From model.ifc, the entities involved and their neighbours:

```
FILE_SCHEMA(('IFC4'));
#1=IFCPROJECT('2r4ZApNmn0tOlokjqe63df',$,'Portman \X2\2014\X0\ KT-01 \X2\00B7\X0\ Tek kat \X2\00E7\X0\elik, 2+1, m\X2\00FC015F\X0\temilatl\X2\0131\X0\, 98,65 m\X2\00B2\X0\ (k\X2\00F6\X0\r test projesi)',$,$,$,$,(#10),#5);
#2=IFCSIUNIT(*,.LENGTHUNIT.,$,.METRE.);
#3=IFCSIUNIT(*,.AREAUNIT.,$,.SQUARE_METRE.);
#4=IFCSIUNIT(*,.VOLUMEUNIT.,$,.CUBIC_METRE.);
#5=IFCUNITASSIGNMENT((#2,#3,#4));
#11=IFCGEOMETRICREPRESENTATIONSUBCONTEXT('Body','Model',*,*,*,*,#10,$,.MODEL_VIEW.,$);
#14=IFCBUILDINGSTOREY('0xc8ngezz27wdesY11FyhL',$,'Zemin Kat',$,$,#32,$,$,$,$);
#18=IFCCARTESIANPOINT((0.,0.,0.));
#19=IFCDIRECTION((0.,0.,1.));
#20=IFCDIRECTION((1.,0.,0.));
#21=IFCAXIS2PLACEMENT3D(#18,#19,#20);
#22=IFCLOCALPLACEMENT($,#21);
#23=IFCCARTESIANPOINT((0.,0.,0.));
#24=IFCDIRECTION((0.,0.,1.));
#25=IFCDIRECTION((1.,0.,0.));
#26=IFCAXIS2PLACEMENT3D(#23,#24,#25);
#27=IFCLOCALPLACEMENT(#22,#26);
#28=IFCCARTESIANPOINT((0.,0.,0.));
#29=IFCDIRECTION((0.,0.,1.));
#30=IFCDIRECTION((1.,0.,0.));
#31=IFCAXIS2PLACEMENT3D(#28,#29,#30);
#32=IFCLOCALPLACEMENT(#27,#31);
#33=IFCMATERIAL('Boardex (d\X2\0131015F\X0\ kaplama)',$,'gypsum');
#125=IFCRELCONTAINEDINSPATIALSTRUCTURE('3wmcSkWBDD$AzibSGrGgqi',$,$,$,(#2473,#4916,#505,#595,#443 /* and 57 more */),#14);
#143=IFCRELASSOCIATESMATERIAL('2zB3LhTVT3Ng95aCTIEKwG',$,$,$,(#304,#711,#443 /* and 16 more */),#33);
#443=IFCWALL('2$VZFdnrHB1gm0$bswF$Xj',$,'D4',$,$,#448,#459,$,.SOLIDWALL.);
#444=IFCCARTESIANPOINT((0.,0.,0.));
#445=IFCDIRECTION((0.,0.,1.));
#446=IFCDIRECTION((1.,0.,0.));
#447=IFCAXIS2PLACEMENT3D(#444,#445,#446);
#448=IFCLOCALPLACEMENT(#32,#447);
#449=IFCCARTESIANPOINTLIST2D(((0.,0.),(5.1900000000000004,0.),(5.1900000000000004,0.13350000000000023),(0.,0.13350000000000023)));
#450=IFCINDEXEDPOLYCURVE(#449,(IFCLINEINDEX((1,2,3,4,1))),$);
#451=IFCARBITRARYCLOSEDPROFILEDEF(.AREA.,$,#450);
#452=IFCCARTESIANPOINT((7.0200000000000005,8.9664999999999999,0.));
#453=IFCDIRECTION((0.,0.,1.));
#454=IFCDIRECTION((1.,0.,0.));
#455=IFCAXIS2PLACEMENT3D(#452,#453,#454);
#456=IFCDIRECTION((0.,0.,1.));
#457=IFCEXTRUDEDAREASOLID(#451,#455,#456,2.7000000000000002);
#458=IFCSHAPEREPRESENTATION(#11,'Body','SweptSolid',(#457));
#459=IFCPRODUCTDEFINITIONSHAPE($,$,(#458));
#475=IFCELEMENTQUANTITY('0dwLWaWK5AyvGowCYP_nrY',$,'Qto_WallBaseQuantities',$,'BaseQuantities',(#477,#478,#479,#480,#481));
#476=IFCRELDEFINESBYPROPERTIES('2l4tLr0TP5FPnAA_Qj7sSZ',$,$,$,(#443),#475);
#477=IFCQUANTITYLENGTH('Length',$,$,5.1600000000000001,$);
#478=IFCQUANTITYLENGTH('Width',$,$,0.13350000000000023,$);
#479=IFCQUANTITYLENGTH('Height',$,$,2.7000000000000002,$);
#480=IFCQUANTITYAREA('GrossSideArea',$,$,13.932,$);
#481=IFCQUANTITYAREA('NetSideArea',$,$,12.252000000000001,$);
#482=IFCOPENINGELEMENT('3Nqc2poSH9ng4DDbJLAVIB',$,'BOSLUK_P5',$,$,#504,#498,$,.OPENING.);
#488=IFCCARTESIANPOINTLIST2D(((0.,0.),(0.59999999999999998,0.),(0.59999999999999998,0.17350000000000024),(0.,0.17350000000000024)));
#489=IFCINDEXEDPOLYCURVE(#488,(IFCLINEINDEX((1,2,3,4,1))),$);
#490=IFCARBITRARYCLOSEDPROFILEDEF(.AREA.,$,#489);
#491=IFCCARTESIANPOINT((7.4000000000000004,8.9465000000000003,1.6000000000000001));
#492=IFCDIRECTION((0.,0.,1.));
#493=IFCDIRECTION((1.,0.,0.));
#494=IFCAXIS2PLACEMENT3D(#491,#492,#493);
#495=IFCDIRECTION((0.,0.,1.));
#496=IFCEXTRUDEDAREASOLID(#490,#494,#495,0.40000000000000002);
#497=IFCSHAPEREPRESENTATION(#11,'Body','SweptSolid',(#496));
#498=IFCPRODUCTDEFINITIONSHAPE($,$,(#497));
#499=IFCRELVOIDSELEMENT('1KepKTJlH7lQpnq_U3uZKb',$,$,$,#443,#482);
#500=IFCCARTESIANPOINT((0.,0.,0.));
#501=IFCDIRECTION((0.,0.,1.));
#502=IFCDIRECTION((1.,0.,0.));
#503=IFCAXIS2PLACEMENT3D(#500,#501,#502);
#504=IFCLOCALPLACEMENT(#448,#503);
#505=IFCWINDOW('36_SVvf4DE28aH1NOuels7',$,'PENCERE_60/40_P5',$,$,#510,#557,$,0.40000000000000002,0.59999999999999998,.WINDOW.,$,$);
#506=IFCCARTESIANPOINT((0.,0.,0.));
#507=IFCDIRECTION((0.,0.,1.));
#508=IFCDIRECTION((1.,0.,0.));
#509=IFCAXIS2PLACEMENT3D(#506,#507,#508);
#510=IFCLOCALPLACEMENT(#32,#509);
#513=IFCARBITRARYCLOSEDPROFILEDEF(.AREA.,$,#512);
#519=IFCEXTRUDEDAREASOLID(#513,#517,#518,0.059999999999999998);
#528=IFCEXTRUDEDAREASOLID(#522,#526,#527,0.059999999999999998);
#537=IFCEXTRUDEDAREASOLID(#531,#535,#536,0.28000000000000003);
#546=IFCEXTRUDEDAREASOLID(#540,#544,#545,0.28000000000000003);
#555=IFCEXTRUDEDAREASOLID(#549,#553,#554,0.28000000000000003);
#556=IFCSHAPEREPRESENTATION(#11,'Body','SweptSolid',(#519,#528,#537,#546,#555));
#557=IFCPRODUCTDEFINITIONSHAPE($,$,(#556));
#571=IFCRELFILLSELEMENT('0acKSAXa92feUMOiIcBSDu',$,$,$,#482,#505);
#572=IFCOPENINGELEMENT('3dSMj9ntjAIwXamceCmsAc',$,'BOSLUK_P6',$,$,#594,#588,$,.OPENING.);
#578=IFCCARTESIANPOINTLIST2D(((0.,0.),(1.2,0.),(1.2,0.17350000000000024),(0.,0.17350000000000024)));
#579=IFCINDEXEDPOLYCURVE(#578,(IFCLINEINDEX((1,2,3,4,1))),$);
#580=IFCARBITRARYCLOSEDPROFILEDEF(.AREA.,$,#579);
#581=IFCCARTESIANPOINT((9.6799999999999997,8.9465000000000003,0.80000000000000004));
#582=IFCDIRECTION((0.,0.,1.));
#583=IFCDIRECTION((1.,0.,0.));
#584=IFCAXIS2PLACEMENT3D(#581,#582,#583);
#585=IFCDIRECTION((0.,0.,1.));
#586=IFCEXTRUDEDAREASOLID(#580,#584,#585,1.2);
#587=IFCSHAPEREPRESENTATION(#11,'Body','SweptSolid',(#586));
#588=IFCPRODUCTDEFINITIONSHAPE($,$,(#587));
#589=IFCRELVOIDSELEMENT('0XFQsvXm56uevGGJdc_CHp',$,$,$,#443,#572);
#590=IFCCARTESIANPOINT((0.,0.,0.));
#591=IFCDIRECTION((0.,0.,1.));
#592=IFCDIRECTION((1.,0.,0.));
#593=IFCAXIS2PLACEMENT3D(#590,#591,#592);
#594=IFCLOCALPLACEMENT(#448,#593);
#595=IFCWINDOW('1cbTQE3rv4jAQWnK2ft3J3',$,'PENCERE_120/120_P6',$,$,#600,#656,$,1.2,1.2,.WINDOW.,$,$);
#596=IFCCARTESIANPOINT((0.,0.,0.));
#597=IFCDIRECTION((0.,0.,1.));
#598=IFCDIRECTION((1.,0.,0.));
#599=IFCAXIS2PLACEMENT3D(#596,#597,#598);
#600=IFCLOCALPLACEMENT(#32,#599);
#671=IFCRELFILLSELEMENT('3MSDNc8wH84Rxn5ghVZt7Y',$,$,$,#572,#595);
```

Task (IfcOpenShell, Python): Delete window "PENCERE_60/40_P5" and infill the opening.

```python
import ifcopenshell
import ifcopenshell.api.feature
import ifcopenshell.api.pset
import ifcopenshell.api.root
import ifcopenshell.geom
import ifcopenshell.util.element
import ifcopenshell.util.shape
import ifcopenshell.util.unit

model = ifcopenshell.open("model.ifc")
area_scale = ifcopenshell.util.unit.calculate_unit_scale(model, "AREAUNIT")
settings = ifcopenshell.geom.settings()


def volume(element):
    """Net volume in cubic metres, openings subtracted."""
    shape = ifcopenshell.geom.create_shape(settings, element)
    return ifcopenshell.util.shape.get_volume(shape.geometry)


window = model.by_guid("36_SVvf4DE28aH1NOuels7")
opening = window.FillsVoids[0].RelatingOpeningElement
wall = opening.VoidsElements[0].RelatingBuildingElement
before = volume(wall)

ifcopenshell.api.root.remove_product(model, product=window)
ifcopenshell.api.feature.remove_feature(model, feature=opening)

after = volume(wall)
thickness = 0.1335  # wall thickness in metres

# Update the wall's stored quantities.
qto = model.by_id(ifcopenshell.util.element.get_pset(wall, "Qto_WallBaseQuantities", should_inherit=False)["id"])
ifcopenshell.api.pset.edit_qto(model, qto=qto, properties={"NetSideArea": after / thickness / area_scale})

print(f"wall volume {before:.3f} -> {after:.3f} m3")

model.write("model_rev.ifc")
```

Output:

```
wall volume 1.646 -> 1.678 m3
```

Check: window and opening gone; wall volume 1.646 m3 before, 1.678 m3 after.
